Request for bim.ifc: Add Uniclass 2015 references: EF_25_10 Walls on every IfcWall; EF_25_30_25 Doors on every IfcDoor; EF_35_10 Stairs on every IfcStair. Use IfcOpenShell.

First a look at what the model holds.

```python
import ifcopenshell

model = ifcopenshell.open("bim.ifc")
print(model.schema)
print("classifications:", [c.Name for c in model.by_type("IfcClassification")])
for ifc_class in ("IfcDoor", "IfcRoof", "IfcStair", "IfcWall", "IfcWindow"):
    print(ifc_class, len(model.by_type(ifc_class)))
```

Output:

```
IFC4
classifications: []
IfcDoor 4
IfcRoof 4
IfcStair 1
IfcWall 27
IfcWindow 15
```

```python
import ifcopenshell
import ifcopenshell.api.classification

model = ifcopenshell.open("bim.ifc")

system = ifcopenshell.api.classification.add_classification(model, classification="Uniclass 2015")

codes = {
    "IfcWall": ("EF_25_10", "Walls"),
    "IfcDoor": ("EF_25_30_25", "Doors"),
    "IfcStair": ("EF_35_10", "Stairs"),
}
for ifc_class, (code, name) in codes.items():
    products = model.by_type(ifc_class)
    ifcopenshell.api.classification.add_reference(
        model, products=products, classification=system, identification=code, name=name
    )
    print(code, len(products))

model.write("bim_updated.ifc")
```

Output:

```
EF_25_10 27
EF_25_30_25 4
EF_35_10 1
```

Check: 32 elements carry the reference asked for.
